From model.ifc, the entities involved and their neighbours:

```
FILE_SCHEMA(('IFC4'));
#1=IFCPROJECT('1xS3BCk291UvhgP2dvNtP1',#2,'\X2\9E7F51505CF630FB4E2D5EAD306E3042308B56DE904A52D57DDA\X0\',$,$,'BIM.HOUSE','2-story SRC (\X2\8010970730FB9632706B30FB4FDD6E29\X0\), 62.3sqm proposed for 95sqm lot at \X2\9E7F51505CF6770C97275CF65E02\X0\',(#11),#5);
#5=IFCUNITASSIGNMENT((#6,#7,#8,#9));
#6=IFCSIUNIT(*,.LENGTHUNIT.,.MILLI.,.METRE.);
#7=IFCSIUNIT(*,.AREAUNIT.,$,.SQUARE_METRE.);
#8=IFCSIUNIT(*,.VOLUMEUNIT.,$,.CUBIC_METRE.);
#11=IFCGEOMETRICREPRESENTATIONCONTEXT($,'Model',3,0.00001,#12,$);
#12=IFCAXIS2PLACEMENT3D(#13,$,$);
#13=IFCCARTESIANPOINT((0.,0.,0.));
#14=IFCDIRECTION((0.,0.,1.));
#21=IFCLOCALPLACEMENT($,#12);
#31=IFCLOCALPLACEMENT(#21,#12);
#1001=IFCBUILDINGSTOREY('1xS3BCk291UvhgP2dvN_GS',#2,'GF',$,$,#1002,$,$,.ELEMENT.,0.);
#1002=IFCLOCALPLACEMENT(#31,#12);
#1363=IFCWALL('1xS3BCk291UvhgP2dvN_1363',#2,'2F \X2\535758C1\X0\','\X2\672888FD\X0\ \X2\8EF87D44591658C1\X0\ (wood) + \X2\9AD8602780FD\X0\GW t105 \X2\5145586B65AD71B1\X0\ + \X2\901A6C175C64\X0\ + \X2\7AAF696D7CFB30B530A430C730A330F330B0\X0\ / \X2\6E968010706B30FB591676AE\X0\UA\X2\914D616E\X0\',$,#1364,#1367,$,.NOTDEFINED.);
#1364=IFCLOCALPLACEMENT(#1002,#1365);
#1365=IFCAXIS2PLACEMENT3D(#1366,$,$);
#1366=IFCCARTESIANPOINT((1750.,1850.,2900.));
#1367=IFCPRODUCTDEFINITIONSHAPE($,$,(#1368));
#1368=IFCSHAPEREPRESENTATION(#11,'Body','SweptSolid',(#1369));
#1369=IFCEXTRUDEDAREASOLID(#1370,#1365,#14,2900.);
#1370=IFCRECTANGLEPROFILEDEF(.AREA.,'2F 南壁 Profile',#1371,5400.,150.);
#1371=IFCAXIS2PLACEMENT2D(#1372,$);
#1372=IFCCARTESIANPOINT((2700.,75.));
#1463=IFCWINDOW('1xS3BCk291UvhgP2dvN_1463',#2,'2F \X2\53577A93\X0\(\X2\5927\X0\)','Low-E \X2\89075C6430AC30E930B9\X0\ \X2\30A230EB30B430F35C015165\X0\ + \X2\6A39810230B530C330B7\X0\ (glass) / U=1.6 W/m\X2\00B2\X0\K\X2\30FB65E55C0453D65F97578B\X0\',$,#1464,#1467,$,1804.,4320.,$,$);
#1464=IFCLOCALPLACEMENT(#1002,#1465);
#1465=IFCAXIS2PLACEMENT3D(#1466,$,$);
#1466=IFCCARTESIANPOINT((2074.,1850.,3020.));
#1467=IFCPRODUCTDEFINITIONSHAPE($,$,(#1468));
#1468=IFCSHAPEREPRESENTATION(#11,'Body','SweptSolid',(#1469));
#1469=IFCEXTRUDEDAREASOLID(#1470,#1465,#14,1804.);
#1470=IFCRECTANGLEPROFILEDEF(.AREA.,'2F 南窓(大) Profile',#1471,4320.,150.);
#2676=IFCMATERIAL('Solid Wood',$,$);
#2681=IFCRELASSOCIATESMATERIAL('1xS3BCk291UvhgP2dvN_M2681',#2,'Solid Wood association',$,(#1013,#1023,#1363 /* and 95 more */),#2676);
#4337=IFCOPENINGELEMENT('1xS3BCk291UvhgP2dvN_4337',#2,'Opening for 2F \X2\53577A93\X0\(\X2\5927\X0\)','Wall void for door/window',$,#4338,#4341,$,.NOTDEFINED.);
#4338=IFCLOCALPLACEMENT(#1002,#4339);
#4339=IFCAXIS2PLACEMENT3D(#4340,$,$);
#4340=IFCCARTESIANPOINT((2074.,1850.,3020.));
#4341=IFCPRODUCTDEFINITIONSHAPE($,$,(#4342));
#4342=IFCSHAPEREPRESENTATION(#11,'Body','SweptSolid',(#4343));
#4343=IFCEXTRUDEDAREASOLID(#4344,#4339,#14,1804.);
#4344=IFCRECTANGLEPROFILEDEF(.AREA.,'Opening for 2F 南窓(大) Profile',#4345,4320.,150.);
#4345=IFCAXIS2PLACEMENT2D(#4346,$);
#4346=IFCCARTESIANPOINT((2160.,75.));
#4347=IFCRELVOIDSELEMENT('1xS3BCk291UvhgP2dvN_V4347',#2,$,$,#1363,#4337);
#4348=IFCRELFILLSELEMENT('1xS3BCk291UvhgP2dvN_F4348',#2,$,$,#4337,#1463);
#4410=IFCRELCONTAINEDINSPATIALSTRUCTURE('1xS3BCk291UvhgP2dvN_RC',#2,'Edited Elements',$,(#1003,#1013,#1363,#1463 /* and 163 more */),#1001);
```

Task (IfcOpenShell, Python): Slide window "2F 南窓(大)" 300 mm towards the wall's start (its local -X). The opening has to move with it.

```python
import ifcopenshell
import ifcopenshell.api.geometry
import ifcopenshell.util.placement

model = ifcopenshell.open("model.ifc")

window = model.by_guid("1xS3BCk291UvhgP2dvN_1463")
opening = window.FillsVoids[0].RelatingOpeningElement
wall = opening.VoidsElements[0].RelatingBuildingElement

wall_matrix = ifcopenshell.util.placement.get_local_placement(wall.ObjectPlacement)
shift = wall_matrix[:3, 0] * -300.0
before = ifcopenshell.util.placement.get_local_placement(window.ObjectPlacement)[:3, 3].copy()

# The window is not placed relative to its opening, so move both.
for product in (opening, window):
    matrix = ifcopenshell.util.placement.get_local_placement(product.ObjectPlacement)
    matrix[:3, 3] += shift
    ifcopenshell.api.geometry.edit_object_placement(model, product=product, matrix=matrix, is_si=False)

after = ifcopenshell.util.placement.get_local_placement(window.ObjectPlacement)[:3, 3]
print("window moved by", (after - before).round(3) + 0.0)

model.write("model_rev.ifc")
```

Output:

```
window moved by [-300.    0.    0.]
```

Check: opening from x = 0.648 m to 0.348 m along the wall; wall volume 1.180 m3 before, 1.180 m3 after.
